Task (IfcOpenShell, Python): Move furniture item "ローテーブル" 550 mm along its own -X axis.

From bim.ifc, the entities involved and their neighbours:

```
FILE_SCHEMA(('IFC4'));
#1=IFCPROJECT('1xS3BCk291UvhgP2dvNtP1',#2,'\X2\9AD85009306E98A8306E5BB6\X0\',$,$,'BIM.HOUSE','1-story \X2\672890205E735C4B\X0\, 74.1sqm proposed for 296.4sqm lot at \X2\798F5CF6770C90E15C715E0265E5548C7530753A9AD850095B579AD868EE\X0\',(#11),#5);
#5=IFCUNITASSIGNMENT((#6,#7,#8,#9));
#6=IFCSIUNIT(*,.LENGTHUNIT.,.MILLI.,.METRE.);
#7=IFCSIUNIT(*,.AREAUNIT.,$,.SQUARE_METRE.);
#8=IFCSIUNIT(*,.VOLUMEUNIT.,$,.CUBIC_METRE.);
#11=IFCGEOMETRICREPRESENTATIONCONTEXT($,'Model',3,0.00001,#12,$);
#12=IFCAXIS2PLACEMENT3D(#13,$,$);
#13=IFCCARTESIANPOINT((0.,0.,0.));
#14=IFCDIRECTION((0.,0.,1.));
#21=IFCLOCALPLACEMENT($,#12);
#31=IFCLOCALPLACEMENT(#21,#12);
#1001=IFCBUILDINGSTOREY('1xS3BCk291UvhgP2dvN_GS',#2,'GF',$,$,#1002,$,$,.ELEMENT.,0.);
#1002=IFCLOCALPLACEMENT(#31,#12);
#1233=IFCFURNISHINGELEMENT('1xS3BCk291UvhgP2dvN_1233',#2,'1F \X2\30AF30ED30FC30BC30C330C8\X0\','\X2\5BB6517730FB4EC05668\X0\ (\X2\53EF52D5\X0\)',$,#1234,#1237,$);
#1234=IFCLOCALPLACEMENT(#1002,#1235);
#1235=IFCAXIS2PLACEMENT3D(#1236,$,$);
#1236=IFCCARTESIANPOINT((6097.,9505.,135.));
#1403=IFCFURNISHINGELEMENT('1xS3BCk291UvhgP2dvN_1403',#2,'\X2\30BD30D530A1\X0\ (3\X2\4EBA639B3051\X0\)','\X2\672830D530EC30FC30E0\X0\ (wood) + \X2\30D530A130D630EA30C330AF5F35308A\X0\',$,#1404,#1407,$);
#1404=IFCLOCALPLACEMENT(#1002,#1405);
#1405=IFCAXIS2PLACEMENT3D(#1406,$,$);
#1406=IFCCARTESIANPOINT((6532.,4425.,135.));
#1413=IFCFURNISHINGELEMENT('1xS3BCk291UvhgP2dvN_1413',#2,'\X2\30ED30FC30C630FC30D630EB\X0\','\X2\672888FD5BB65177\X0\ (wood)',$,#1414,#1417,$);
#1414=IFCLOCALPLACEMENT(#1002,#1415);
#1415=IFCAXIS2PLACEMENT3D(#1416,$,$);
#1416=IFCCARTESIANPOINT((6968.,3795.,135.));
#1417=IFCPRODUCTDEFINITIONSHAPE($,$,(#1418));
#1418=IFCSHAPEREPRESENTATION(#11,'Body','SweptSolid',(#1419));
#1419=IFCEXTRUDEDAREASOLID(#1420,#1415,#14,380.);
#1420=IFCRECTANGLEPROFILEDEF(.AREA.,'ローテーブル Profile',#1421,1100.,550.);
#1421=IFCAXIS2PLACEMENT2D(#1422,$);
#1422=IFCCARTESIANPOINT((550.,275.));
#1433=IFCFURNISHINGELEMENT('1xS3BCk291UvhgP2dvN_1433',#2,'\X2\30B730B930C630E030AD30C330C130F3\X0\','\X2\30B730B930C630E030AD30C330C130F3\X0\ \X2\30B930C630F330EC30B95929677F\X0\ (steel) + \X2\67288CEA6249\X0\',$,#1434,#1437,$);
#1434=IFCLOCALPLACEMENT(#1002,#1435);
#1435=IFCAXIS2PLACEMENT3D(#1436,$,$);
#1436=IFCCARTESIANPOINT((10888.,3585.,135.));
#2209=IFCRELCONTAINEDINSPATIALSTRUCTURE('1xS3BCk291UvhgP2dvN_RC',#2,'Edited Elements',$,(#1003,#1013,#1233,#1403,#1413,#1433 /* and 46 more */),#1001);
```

```python
import ifcopenshell
import ifcopenshell.api.geometry
import ifcopenshell.util.placement

model = ifcopenshell.open("bim.ifc")

item = model.by_guid("1xS3BCk291UvhgP2dvN_1413")
matrix = ifcopenshell.util.placement.get_local_placement(item.ObjectPlacement)
matrix[:3, 3] -= matrix[:3, 0] * 550.0
ifcopenshell.api.geometry.edit_object_placement(model, product=item, matrix=matrix, is_si=False)

print(ifcopenshell.util.placement.get_local_placement(item.ObjectPlacement).round(3) + 0.0)

model.write("bim-out.ifc")
```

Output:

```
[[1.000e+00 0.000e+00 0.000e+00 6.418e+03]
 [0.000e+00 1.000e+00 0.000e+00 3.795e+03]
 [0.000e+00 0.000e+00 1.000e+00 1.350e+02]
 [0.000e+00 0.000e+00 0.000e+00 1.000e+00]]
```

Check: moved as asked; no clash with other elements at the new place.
